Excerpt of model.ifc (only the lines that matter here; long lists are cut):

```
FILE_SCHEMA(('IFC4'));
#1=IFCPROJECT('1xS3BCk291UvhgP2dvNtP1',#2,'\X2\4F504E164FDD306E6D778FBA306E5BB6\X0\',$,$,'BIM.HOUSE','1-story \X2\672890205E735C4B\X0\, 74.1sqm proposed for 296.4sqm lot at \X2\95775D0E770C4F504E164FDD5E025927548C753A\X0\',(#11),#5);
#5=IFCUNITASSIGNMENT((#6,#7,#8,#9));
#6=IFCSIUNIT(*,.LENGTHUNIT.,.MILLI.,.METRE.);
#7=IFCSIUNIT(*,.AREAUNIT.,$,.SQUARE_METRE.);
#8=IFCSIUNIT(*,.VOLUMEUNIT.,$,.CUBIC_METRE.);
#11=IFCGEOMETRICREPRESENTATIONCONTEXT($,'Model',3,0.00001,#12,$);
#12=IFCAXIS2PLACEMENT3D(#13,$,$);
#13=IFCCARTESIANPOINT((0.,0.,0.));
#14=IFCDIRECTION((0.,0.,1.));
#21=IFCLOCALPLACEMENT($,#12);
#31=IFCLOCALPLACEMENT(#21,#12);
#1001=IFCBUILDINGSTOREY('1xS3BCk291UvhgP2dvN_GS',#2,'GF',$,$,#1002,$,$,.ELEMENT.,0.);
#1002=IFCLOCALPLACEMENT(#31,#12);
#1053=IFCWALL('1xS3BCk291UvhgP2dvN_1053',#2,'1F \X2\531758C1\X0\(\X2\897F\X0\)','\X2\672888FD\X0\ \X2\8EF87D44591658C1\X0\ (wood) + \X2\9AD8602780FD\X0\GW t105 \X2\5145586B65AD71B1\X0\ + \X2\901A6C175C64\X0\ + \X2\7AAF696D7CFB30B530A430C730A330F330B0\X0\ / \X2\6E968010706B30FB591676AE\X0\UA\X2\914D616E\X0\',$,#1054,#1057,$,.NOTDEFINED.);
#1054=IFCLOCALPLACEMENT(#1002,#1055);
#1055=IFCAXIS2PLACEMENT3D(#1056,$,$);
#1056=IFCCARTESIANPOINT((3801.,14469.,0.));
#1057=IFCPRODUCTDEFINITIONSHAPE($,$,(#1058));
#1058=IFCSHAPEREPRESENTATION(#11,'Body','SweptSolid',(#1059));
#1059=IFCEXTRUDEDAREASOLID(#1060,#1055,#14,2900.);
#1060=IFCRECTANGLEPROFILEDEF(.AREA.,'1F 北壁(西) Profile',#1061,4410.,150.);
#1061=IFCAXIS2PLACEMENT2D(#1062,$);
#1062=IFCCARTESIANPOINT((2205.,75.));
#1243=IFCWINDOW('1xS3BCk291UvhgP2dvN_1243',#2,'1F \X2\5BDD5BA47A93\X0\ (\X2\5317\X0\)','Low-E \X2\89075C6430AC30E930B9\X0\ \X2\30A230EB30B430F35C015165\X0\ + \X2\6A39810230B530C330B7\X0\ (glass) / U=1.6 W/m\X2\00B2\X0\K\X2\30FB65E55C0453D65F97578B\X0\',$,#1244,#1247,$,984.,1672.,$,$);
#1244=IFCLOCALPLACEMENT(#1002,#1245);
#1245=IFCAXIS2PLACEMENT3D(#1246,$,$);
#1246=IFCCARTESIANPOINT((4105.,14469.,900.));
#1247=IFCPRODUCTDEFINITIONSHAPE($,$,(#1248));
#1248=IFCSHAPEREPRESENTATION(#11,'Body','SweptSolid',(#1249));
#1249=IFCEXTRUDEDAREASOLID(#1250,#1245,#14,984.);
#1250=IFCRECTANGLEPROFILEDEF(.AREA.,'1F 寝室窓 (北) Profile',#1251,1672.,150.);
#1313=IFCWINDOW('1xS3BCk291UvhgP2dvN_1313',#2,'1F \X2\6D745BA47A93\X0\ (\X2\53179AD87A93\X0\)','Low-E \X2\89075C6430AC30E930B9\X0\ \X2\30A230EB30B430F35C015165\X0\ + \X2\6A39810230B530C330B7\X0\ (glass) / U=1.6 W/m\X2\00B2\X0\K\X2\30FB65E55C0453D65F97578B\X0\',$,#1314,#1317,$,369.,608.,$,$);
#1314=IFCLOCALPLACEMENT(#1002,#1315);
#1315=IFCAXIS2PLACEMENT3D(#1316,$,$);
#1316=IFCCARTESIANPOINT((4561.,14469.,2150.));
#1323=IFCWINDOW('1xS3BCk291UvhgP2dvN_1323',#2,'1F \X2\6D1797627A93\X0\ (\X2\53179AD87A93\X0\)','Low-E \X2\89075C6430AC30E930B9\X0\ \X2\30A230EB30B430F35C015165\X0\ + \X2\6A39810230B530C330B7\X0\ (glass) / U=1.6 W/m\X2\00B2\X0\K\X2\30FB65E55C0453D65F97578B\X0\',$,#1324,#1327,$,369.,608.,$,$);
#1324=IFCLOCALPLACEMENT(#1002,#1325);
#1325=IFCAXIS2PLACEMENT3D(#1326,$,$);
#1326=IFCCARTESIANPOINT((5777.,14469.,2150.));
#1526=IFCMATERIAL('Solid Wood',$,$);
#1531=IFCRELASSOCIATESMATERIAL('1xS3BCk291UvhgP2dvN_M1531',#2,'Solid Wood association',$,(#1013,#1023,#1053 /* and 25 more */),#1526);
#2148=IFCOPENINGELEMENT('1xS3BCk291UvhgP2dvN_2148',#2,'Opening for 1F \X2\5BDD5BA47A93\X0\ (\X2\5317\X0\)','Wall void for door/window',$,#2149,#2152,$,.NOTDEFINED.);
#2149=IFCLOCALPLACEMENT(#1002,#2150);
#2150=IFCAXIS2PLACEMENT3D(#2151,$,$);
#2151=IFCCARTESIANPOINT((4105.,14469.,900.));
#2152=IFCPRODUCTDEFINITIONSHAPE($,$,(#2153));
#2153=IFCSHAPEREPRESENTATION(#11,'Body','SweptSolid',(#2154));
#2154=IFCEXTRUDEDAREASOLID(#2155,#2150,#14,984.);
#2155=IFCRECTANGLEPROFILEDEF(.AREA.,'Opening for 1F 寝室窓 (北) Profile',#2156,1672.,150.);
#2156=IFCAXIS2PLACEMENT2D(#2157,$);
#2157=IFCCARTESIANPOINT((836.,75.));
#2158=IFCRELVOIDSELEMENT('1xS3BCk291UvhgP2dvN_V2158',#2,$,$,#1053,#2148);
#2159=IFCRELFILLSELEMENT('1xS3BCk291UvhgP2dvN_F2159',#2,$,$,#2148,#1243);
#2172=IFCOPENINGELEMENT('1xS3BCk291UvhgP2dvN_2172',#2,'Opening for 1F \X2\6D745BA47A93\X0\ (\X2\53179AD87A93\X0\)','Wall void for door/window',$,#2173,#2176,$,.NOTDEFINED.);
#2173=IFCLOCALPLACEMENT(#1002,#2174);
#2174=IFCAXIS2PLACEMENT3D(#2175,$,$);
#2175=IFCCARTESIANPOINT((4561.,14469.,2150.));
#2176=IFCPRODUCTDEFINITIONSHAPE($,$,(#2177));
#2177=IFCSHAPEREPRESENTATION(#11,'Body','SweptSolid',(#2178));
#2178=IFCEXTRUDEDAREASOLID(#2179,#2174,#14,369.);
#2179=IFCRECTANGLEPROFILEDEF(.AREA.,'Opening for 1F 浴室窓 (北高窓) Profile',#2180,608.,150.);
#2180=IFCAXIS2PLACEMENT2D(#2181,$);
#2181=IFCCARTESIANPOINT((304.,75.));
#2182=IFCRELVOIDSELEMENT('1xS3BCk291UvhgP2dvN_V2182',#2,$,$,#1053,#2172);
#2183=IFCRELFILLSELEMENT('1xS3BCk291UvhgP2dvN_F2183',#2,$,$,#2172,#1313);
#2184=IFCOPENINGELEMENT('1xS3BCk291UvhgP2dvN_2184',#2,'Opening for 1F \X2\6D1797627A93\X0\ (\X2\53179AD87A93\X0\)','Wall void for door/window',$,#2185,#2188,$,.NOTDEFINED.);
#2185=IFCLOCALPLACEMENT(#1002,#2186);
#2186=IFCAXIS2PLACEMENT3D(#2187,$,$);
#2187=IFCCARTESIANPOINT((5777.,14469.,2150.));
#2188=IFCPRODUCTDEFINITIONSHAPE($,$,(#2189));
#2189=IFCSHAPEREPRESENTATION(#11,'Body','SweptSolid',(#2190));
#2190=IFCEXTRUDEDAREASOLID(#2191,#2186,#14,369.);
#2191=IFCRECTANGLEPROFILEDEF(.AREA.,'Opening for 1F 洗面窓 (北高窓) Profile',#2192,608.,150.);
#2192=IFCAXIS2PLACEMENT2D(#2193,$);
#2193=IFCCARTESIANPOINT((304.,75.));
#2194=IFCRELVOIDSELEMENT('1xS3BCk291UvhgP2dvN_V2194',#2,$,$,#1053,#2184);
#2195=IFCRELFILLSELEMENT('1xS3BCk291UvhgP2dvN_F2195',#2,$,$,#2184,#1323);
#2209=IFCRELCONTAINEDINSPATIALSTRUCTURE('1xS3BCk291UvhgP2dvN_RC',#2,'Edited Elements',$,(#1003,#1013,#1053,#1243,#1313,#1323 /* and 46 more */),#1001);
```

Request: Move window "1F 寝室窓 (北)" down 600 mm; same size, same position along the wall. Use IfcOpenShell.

```python
import numpy as np
import ifcopenshell
import ifcopenshell.api.geometry
import ifcopenshell.util.placement
import ifcopenshell.util.unit

model = ifcopenshell.open("model.ifc")
unit_scale = ifcopenshell.util.unit.calculate_unit_scale(model)

window = model.by_id(1243)
opening = window.FillsVoids[0].RelatingOpeningElement
dz = -600.0

shift = np.array([0.0, 0.0, dz])
# The window is not placed relative to its opening, so move both.
for product in (opening, window):
    matrix = ifcopenshell.util.placement.get_local_placement(product.ObjectPlacement)
    matrix[:3, 3] += shift
    ifcopenshell.api.geometry.edit_object_placement(model, product=product, matrix=matrix, is_si=False)

print(f"moved by {dz * unit_scale:+.3f} m")

model.write("model_updated.ifc")
```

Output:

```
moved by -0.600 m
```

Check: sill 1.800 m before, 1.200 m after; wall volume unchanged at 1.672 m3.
